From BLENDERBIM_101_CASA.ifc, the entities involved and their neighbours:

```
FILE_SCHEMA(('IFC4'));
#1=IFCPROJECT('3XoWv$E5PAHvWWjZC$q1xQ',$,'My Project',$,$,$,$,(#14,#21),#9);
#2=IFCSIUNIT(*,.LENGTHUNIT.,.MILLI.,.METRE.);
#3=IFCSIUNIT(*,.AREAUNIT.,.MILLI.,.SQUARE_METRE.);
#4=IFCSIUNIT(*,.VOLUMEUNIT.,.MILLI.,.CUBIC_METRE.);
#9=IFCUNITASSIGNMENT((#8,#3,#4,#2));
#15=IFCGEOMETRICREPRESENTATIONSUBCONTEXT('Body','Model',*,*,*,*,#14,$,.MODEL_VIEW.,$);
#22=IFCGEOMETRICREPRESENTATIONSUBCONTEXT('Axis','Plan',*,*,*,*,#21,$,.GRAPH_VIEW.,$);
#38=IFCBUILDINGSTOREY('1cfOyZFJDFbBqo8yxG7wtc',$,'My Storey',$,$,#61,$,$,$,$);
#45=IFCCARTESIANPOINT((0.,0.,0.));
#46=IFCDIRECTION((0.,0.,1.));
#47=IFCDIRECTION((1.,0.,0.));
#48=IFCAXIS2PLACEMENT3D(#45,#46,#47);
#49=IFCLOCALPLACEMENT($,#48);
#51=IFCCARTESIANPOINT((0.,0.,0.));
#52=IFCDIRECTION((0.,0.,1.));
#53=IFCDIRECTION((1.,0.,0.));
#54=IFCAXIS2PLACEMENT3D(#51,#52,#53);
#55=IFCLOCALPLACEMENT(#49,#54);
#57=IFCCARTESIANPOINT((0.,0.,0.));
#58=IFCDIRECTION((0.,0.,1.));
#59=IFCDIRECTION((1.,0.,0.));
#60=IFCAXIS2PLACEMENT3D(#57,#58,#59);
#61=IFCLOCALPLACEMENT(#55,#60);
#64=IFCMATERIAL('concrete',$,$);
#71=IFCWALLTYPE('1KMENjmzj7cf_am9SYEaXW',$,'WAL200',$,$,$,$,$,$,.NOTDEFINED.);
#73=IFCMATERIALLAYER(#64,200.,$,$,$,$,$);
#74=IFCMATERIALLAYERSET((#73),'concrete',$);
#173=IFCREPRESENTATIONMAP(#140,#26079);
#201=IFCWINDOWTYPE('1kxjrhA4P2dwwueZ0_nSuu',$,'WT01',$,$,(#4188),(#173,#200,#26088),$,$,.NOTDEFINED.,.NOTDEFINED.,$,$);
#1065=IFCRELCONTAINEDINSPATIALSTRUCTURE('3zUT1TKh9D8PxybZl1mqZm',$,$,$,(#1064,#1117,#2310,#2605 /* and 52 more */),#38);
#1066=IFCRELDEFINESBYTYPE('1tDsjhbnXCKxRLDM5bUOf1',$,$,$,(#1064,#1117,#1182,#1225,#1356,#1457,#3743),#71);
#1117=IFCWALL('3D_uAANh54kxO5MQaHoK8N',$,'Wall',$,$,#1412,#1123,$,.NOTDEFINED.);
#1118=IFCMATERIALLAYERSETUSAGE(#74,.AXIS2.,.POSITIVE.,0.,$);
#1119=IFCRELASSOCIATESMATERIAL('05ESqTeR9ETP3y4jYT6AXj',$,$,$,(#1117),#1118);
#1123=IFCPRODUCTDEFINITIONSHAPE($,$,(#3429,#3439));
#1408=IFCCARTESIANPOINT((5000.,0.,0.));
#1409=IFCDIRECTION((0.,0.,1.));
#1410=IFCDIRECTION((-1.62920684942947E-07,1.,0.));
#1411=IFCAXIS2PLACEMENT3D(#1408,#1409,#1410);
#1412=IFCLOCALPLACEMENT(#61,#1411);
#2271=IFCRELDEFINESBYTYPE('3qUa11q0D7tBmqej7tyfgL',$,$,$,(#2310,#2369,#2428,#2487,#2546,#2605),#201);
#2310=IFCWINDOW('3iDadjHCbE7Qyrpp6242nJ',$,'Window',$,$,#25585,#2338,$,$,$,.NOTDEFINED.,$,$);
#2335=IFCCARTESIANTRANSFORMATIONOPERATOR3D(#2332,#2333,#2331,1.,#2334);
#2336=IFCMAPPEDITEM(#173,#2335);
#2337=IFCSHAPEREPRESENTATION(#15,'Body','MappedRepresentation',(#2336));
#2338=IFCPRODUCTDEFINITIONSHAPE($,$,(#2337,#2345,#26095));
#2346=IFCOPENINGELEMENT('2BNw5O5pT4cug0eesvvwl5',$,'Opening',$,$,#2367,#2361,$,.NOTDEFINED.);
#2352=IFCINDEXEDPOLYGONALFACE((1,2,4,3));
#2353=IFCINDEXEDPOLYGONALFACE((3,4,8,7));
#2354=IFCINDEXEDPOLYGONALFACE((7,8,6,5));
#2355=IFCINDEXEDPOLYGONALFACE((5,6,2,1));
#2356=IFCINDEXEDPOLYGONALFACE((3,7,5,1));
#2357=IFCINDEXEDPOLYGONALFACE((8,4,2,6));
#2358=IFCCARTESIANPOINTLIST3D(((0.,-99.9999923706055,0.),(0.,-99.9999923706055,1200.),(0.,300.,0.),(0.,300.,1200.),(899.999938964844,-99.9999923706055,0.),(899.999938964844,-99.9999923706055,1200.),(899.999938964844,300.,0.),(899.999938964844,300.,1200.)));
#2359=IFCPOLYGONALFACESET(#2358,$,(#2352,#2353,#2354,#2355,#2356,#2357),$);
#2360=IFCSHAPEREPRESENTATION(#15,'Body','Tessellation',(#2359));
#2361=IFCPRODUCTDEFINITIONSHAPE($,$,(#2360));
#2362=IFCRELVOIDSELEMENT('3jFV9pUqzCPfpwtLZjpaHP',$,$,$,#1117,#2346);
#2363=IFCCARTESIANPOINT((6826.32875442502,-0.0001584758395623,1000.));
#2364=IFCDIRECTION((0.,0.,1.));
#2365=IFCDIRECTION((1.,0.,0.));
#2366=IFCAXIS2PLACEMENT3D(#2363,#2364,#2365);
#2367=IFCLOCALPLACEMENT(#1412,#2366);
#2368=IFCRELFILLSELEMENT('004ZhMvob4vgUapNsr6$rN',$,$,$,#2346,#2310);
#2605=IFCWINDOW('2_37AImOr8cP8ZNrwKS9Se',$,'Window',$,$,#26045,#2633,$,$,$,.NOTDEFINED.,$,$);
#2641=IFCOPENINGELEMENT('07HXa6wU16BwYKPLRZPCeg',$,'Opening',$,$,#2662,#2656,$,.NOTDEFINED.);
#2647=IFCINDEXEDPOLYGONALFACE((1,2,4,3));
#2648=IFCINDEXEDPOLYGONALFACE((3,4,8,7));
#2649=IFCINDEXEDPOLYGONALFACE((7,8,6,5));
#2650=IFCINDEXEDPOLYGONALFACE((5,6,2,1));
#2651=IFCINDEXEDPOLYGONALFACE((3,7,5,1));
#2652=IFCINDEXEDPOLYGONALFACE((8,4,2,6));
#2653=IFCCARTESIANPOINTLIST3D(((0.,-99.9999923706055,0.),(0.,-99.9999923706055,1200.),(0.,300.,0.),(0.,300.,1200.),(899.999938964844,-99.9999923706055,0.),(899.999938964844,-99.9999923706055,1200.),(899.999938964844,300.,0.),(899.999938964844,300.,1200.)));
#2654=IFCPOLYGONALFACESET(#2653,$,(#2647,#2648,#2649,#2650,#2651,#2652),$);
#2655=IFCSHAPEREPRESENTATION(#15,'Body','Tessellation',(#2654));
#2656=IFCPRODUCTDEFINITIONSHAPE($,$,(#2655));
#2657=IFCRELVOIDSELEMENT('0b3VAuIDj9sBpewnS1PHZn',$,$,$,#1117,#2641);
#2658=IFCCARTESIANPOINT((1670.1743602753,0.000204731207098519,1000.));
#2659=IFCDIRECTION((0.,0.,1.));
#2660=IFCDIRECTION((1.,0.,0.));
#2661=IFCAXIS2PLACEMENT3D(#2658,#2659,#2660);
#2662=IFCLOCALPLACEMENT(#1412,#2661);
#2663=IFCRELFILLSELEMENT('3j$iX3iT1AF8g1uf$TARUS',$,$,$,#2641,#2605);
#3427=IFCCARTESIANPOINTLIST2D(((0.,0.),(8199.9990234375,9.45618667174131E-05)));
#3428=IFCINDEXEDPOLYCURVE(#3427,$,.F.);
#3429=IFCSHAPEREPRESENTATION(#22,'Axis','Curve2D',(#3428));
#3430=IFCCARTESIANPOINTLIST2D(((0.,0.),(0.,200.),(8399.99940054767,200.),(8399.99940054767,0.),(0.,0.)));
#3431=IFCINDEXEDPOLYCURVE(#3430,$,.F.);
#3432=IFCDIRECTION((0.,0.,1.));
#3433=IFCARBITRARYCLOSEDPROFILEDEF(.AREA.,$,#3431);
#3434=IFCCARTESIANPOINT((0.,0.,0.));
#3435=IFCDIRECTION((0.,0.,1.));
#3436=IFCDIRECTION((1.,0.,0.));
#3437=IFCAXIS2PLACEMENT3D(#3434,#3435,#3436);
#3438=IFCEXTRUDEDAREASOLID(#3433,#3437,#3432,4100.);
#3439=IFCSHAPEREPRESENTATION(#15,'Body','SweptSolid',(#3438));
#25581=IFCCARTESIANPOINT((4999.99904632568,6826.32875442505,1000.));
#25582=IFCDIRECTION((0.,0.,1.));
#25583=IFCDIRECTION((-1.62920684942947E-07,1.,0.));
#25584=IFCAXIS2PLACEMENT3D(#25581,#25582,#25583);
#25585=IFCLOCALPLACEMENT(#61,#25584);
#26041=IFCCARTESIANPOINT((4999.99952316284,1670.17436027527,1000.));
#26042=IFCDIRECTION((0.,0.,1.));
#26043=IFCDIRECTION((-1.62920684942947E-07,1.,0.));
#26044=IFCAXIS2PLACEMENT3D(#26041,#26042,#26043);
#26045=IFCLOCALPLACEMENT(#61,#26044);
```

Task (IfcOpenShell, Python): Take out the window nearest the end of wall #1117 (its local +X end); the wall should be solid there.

```python
import ifcopenshell
import ifcopenshell.api.feature
import ifcopenshell.api.root
import ifcopenshell.geom
import ifcopenshell.util.shape

model = ifcopenshell.open("BLENDERBIM_101_CASA.ifc")
settings = ifcopenshell.geom.settings()


def volume(element):
    """Net volume in cubic metres, openings subtracted."""
    shape = ifcopenshell.geom.create_shape(settings, element)
    return ifcopenshell.util.shape.get_volume(shape.geometry)


window = model.by_id(2310)
opening = window.FillsVoids[0].RelatingOpeningElement
wall = opening.VoidsElements[0].RelatingBuildingElement
before = volume(wall)

ifcopenshell.api.root.remove_product(model, product=window)
ifcopenshell.api.feature.remove_feature(model, feature=opening)

after = volume(wall)

print(f"wall volume {before:.3f} -> {after:.3f} m3")

model.write("BLENDERBIM_101_CASA_updated.ifc")
```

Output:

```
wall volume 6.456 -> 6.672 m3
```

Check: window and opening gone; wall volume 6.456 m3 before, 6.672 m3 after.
